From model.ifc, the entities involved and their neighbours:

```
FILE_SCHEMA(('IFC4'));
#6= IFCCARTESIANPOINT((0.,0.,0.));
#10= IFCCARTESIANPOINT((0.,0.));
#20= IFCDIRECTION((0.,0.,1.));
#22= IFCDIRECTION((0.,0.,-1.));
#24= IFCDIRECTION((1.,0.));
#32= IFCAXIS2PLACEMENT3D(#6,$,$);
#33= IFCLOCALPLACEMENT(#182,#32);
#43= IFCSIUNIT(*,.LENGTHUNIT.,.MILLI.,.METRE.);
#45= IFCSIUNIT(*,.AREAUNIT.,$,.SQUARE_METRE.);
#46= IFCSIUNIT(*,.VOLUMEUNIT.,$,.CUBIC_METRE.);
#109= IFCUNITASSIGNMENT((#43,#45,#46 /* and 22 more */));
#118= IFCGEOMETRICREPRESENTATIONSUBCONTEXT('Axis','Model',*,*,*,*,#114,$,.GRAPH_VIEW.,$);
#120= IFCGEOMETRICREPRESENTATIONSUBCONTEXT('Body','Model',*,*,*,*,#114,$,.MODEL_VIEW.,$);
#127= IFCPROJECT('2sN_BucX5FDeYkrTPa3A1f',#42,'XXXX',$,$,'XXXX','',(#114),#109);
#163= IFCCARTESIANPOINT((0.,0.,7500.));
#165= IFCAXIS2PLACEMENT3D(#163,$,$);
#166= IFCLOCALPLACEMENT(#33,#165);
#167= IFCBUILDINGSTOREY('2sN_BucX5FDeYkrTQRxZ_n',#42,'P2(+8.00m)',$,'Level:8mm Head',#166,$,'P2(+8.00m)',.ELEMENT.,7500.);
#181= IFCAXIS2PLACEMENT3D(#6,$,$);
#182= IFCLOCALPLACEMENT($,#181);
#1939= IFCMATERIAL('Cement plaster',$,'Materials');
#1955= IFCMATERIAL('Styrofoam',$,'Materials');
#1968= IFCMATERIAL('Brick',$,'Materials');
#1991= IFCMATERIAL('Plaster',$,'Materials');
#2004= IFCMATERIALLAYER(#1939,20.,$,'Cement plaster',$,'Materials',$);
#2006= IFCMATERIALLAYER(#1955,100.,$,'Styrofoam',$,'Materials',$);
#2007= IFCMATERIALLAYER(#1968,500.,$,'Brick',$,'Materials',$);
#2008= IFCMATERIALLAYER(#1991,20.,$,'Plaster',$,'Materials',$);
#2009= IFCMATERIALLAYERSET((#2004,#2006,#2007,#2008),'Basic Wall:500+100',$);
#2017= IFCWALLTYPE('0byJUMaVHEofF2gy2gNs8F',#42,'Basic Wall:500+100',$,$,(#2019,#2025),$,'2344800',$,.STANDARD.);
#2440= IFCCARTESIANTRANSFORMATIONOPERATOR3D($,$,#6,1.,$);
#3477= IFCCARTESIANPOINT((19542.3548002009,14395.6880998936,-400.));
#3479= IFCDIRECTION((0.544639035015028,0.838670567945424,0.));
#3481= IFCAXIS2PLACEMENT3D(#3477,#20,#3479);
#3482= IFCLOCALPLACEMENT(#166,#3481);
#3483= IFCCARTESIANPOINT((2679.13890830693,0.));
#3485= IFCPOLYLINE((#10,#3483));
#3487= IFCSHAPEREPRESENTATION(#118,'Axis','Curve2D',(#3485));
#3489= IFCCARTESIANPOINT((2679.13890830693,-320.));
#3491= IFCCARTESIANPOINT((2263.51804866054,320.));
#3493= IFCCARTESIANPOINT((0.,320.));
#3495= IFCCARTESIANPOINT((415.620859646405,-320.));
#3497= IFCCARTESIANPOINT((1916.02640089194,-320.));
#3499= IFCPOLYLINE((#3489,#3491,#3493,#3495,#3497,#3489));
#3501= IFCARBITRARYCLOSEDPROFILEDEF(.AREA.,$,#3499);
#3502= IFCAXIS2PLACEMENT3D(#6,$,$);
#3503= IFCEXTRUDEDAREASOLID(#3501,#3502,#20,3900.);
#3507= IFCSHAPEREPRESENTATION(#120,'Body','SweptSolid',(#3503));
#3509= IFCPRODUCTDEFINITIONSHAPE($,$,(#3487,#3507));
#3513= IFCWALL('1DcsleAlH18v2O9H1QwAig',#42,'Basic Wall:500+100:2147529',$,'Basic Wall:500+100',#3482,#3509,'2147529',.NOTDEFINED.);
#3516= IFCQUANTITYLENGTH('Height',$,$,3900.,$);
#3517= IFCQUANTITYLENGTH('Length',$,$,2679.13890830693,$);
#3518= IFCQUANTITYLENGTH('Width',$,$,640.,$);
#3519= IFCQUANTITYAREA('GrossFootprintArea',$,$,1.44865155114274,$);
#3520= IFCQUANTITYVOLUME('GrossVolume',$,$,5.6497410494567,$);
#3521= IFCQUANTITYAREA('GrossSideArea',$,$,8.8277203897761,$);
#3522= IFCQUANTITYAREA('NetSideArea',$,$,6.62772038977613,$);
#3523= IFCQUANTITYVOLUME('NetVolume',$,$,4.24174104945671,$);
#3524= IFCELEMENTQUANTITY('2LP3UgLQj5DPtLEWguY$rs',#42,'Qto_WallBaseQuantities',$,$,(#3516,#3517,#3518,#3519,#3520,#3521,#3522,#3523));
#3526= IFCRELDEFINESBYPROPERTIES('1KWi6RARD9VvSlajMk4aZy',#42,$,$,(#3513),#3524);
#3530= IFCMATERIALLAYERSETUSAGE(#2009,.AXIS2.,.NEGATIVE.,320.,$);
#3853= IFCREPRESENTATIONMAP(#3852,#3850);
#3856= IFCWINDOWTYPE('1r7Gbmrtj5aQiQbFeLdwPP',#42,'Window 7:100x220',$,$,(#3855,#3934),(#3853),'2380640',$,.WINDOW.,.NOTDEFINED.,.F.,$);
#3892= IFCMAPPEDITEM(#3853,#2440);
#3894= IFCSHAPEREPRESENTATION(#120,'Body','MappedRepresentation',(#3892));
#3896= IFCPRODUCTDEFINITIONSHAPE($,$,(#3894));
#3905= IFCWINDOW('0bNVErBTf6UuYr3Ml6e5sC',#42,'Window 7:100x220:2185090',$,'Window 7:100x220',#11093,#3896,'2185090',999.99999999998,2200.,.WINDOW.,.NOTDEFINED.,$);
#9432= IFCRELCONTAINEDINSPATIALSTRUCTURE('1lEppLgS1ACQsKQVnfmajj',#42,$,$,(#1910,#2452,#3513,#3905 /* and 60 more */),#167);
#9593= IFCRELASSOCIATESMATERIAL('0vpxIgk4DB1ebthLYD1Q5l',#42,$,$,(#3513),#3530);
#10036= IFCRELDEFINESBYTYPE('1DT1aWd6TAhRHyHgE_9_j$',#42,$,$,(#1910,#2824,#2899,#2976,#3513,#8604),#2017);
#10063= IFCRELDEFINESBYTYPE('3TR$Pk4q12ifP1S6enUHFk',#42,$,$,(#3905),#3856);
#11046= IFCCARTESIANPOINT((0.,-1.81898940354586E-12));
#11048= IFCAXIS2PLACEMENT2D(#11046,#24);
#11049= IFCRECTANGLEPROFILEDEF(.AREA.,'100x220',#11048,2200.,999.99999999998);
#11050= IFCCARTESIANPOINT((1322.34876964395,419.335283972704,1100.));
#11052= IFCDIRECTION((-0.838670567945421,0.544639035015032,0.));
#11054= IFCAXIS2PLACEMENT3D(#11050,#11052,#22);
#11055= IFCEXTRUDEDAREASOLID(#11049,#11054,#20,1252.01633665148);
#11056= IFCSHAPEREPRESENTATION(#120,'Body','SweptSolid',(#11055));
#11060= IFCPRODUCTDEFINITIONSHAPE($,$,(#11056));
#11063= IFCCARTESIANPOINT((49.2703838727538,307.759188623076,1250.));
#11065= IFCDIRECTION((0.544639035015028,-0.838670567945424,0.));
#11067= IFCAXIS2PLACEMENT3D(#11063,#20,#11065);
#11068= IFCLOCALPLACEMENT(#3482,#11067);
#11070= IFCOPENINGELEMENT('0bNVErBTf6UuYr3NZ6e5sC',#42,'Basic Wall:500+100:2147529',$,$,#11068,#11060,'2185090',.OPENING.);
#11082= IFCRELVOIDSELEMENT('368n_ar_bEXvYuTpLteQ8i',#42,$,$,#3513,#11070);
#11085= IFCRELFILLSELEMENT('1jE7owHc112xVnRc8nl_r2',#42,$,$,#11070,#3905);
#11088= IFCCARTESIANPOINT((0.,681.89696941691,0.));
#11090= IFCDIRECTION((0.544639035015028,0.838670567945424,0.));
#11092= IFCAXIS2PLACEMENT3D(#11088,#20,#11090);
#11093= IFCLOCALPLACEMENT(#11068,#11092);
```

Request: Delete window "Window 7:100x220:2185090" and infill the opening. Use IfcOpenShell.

```python
import ifcopenshell
import ifcopenshell.api.feature
import ifcopenshell.api.pset
import ifcopenshell.api.root
import ifcopenshell.geom
import ifcopenshell.util.element
import ifcopenshell.util.shape
import ifcopenshell.util.unit

model = ifcopenshell.open("model.ifc")
area_scale = ifcopenshell.util.unit.calculate_unit_scale(model, "AREAUNIT")
volume_scale = ifcopenshell.util.unit.calculate_unit_scale(model, "VOLUMEUNIT")
settings = ifcopenshell.geom.settings()


def volume(element):
    """Net volume in cubic metres, openings subtracted."""
    shape = ifcopenshell.geom.create_shape(settings, element)
    return ifcopenshell.util.shape.get_volume(shape.geometry)


window = model.by_id(3905)
opening = window.FillsVoids[0].RelatingOpeningElement
wall = opening.VoidsElements[0].RelatingBuildingElement
before = volume(wall)

ifcopenshell.api.root.remove_product(model, product=window)
ifcopenshell.api.feature.remove_feature(model, feature=opening)

after = volume(wall)
thickness = 0.64  # wall thickness in metres

# Update the wall's stored quantities.
qto = model.by_id(ifcopenshell.util.element.get_pset(wall, "Qto_WallBaseQuantities", should_inherit=False)["id"])
ifcopenshell.api.pset.edit_qto(model, qto=qto, properties={
    "NetSideArea": after / thickness / area_scale,
    "NetVolume": after / volume_scale,
})

print(f"wall volume {before:.3f} -> {after:.3f} m3")

model.write("model-out.ifc")
```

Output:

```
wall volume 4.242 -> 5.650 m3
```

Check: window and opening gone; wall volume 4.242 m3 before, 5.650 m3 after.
